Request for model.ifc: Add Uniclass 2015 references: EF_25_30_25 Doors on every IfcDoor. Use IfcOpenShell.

First a look at what the model holds.

```python
import ifcopenshell

model = ifcopenshell.open("model.ifc")
print(model.schema)
print("classifications:", [c.Name for c in model.by_type("IfcClassification")])
for ifc_class in ("IfcDoor", "IfcRoof", "IfcStair", "IfcWall", "IfcWindow"):
    print(ifc_class, len(model.by_type(ifc_class)))
```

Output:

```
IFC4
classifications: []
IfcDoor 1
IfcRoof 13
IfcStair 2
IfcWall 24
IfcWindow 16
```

```python
import ifcopenshell
import ifcopenshell.api.classification

model = ifcopenshell.open("model.ifc")

system = ifcopenshell.api.classification.add_classification(model, classification="Uniclass 2015")

codes = {
    "IfcDoor": ("EF_25_30_25", "Doors"),
}
for ifc_class, (code, name) in codes.items():
    products = model.by_type(ifc_class)
    ifcopenshell.api.classification.add_reference(
        model, products=products, classification=system, identification=code, name=name
    )
    print(code, len(products))

model.write("model-out.ifc")
```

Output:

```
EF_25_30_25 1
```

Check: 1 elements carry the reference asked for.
